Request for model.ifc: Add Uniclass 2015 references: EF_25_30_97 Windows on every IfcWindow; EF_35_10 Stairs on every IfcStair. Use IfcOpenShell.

First a look at what the model holds.

```python
import ifcopenshell

model = ifcopenshell.open("model.ifc")
print(model.schema)
print("classifications:", [c.Name for c in model.by_type("IfcClassification")])
for ifc_class in ("IfcDoor", "IfcRoof", "IfcStair", "IfcWall", "IfcWindow"):
    print(ifc_class, len(model.by_type(ifc_class)))
```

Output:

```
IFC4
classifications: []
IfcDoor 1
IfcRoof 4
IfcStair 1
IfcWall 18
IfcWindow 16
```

```python
import ifcopenshell
import ifcopenshell.api.classification

model = ifcopenshell.open("model.ifc")

system = ifcopenshell.api.classification.add_classification(model, classification="Uniclass 2015")

codes = {
    "IfcWindow": ("EF_25_30_97", "Windows"),
    "IfcStair": ("EF_35_10", "Stairs"),
}
for ifc_class, (code, name) in codes.items():
    products = model.by_type(ifc_class)
    ifcopenshell.api.classification.add_reference(
        model, products=products, classification=system, identification=code, name=name
    )
    print(code, len(products))

model.write("model-out.ifc")
```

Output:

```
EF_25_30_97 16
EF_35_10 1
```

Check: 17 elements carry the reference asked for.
